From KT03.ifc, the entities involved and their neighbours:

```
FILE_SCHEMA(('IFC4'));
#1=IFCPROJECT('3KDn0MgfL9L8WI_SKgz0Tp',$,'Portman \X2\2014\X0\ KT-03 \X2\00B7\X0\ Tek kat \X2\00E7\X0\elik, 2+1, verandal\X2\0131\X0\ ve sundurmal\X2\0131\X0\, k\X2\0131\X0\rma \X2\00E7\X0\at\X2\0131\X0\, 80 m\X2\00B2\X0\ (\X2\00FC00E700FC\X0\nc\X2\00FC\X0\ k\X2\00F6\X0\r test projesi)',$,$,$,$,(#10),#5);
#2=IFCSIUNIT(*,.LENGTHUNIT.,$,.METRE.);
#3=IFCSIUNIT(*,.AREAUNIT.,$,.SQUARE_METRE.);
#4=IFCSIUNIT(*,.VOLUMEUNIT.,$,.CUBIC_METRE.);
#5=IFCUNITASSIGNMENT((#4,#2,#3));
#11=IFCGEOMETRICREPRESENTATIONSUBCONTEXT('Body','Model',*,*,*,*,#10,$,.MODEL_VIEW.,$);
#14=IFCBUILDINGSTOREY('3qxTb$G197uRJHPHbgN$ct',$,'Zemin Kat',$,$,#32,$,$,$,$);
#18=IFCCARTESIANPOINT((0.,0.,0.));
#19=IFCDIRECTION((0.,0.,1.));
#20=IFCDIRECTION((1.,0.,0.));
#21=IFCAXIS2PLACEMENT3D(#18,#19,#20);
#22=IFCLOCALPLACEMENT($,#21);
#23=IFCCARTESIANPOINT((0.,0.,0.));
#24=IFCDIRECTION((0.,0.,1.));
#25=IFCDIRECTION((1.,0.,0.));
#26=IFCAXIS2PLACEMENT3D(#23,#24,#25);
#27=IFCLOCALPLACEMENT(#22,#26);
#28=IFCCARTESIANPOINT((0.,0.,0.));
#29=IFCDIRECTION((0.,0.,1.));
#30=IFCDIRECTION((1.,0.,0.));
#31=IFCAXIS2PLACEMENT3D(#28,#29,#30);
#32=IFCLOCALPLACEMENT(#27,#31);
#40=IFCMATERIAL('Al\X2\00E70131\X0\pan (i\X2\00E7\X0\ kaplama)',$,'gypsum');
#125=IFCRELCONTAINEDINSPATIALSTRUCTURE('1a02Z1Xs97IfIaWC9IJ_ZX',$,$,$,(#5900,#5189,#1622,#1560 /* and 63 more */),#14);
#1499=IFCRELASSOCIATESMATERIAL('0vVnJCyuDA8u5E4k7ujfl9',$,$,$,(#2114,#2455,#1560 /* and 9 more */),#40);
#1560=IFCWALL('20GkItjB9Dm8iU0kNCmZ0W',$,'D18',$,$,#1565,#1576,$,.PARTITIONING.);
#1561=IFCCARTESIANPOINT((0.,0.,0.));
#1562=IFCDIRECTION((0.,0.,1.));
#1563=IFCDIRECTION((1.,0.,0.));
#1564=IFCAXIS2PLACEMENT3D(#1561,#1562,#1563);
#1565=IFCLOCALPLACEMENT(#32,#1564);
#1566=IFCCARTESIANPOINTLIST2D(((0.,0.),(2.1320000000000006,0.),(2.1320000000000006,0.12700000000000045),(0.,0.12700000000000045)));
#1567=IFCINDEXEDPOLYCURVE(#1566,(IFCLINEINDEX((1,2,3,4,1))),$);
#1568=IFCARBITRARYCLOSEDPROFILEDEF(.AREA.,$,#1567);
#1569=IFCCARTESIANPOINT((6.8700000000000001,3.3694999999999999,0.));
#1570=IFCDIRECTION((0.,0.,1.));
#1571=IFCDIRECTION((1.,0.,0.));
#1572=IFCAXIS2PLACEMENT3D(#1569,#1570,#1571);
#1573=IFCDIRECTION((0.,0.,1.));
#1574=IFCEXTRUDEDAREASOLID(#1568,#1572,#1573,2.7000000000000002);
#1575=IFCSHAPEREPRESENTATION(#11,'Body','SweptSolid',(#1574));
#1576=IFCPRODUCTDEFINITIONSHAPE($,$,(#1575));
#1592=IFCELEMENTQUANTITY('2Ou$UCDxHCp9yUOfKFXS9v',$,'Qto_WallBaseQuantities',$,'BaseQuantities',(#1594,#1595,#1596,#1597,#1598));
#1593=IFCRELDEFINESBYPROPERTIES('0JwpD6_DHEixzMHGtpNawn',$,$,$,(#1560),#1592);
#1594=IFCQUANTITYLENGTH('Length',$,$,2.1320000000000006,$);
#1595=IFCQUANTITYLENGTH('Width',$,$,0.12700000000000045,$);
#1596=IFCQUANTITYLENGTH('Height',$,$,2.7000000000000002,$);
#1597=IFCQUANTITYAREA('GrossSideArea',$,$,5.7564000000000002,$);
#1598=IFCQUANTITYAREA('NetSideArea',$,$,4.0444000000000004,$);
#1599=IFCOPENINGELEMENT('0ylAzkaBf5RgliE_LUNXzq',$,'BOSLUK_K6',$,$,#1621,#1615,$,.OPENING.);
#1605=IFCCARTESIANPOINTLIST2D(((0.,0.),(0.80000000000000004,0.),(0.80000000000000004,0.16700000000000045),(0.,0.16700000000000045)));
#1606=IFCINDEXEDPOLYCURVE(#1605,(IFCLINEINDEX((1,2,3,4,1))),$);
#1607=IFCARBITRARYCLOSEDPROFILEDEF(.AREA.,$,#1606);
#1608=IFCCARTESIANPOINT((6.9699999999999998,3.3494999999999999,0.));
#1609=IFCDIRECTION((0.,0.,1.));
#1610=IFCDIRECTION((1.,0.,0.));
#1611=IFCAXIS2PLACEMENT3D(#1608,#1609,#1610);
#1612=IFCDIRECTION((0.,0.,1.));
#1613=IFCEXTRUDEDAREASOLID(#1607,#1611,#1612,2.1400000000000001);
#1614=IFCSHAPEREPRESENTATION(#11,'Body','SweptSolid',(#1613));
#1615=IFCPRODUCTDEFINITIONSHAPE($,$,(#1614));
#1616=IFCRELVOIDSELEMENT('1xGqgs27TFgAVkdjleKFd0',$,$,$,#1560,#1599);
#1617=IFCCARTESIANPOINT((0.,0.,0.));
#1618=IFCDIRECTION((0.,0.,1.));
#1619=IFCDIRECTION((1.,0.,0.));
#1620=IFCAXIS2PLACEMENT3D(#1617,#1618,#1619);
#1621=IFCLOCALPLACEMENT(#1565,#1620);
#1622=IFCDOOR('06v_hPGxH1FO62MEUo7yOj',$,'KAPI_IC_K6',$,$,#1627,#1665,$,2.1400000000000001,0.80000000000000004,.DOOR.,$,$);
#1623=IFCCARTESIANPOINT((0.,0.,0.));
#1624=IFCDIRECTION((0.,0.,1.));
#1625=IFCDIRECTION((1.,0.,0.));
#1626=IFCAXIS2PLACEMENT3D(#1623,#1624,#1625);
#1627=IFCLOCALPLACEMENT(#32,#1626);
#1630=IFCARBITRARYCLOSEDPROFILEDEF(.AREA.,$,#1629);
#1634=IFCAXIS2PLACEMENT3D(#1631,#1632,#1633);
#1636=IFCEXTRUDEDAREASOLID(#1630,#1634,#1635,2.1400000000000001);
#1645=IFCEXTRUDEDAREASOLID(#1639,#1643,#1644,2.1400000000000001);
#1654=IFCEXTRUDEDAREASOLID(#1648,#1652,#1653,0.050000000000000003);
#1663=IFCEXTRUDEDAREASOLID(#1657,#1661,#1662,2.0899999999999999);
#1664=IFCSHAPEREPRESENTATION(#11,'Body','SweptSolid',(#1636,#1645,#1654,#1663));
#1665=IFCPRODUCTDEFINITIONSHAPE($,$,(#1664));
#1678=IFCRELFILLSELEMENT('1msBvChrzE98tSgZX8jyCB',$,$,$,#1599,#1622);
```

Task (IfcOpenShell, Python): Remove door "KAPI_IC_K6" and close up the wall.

```python
import ifcopenshell
import ifcopenshell.api.feature
import ifcopenshell.api.pset
import ifcopenshell.api.root
import ifcopenshell.geom
import ifcopenshell.util.element
import ifcopenshell.util.shape
import ifcopenshell.util.unit

model = ifcopenshell.open("KT03.ifc")
area_scale = ifcopenshell.util.unit.calculate_unit_scale(model, "AREAUNIT")
settings = ifcopenshell.geom.settings()


def volume(element):
    """Net volume in cubic metres, openings subtracted."""
    shape = ifcopenshell.geom.create_shape(settings, element)
    return ifcopenshell.util.shape.get_volume(shape.geometry)


door = model.by_guid("06v_hPGxH1FO62MEUo7yOj")
opening = door.FillsVoids[0].RelatingOpeningElement
wall = opening.VoidsElements[0].RelatingBuildingElement
before = volume(wall)

ifcopenshell.api.root.remove_product(model, product=door)
ifcopenshell.api.feature.remove_feature(model, feature=opening)

after = volume(wall)
thickness = 0.127  # wall thickness in metres

# Update the wall's stored quantities.
qto = model.by_id(ifcopenshell.util.element.get_pset(wall, "Qto_WallBaseQuantities", should_inherit=False)["id"])
ifcopenshell.api.pset.edit_qto(model, qto=qto, properties={"NetSideArea": after / thickness / area_scale})

print(f"wall volume {before:.3f} -> {after:.3f} m3")

model.write("KT03_v2.ifc")
```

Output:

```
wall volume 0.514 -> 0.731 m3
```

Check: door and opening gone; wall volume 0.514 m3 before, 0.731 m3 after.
